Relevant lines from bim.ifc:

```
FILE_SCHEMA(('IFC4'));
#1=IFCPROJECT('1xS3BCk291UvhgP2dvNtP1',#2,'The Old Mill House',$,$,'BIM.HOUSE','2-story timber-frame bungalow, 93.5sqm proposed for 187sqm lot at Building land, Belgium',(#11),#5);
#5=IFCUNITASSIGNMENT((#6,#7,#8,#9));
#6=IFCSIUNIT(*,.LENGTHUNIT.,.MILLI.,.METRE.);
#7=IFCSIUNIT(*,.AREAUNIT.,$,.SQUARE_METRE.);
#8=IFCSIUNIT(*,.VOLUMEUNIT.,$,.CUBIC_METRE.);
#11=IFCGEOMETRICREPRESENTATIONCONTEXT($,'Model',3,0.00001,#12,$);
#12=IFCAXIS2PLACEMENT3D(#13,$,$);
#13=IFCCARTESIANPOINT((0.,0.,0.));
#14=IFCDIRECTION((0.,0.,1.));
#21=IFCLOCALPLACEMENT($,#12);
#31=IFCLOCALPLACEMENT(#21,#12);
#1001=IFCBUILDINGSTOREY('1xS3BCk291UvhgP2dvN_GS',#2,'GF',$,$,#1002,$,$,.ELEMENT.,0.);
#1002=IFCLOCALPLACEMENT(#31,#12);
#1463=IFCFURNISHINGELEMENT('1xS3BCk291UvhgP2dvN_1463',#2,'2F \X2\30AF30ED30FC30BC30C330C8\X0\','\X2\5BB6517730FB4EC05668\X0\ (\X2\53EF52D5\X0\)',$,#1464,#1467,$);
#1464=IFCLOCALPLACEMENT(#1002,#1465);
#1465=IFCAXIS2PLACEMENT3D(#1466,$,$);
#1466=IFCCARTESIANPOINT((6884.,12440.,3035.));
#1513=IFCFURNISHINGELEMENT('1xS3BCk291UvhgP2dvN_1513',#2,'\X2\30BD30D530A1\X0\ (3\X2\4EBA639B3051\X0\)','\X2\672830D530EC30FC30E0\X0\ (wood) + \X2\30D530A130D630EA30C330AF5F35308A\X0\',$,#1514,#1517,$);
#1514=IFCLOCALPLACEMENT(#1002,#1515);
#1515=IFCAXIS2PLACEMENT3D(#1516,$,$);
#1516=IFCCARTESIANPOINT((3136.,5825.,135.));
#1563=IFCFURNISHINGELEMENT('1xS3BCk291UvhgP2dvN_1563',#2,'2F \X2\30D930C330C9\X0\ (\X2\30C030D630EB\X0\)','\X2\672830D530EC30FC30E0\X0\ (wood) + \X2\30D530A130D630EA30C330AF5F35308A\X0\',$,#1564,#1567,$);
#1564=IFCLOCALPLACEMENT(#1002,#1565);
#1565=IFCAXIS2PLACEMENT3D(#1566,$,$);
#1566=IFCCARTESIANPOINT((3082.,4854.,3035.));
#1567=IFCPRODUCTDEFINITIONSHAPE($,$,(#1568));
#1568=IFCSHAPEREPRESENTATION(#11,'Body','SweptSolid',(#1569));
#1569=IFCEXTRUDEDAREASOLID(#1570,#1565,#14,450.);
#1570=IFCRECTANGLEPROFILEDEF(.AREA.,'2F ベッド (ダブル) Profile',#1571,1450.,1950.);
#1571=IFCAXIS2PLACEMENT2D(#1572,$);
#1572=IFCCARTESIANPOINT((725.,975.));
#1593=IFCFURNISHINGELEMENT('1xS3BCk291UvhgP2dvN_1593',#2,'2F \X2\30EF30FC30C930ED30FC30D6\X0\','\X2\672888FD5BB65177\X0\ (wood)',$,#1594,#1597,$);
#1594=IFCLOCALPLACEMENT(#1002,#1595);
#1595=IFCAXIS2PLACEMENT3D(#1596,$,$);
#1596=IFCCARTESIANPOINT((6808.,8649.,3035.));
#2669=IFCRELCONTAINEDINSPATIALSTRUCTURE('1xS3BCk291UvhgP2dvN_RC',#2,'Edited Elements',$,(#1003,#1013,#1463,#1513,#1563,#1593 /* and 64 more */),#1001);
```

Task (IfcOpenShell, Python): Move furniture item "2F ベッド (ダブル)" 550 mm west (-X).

```python
import ifcopenshell
import ifcopenshell.api.geometry
import ifcopenshell.util.placement

model = ifcopenshell.open("bim.ifc")

item = model.by_guid("1xS3BCk291UvhgP2dvN_1563")
matrix = ifcopenshell.util.placement.get_local_placement(item.ObjectPlacement)
matrix[0, 3] -= 550.0
ifcopenshell.api.geometry.edit_object_placement(model, product=item, matrix=matrix, is_si=False)

print(ifcopenshell.util.placement.get_local_placement(item.ObjectPlacement).round(3) + 0.0)

model.write("bim_v2.ifc")
```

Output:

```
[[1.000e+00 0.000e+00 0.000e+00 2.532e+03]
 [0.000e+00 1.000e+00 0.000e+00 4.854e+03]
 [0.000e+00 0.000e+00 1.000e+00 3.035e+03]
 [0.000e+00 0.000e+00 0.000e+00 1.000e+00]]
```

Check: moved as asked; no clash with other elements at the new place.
